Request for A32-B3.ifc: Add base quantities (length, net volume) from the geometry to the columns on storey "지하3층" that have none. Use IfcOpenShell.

First a look at what the model holds.

```python
import ifcopenshell
import ifcopenshell.util.element
import ifcopenshell.util.unit

model = ifcopenshell.open("A32-B3.ifc")
print(model.schema)
for unit_type in ("LENGTHUNIT", "AREAUNIT", "VOLUMEUNIT"):
    print(unit_type, ifcopenshell.util.unit.calculate_unit_scale(model, unit_type))
storey = next(s for s in model.by_type("IfcBuildingStorey") if s.Name == "지하3층")
columns = [e for e in ifcopenshell.util.element.get_decomposition(storey) if e.is_a("IfcColumn")]
for e in sorted(columns, key=lambda e: e.id()):
    print(e.id(), e.is_a(), e.Name, list(ifcopenshell.util.element.get_psets(e, qtos_only=True)), sep=" | ")
```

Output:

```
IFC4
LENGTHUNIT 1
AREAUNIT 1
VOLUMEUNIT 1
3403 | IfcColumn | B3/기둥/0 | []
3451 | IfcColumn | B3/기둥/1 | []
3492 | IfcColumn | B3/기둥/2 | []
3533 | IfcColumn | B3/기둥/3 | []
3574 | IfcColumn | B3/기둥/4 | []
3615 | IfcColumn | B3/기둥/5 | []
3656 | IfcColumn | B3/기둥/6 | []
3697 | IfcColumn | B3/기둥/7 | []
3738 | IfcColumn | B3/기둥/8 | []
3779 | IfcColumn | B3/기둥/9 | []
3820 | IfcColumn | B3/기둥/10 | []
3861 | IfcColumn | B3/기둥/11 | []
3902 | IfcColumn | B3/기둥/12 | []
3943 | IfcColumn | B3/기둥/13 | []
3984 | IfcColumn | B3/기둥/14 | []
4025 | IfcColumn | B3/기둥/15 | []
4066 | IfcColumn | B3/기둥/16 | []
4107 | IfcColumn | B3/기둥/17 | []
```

```python
import ifcopenshell
import ifcopenshell.api.pset
import ifcopenshell.geom
import ifcopenshell.util.element
import ifcopenshell.util.shape
import ifcopenshell.util.unit

model = ifcopenshell.open("A32-B3.ifc")
unit_scale = ifcopenshell.util.unit.calculate_unit_scale(model)
volume_scale = ifcopenshell.util.unit.calculate_unit_scale(model, "VOLUMEUNIT")
settings = ifcopenshell.geom.settings()

storey = next(s for s in model.by_type("IfcBuildingStorey") if s.Name == "지하3층")
columns = [e for e in ifcopenshell.util.element.get_decomposition(storey) if e.is_a("IfcColumn")]

for e in sorted(columns, key=lambda e: e.id()):
    if ifcopenshell.util.element.get_psets(e, qtos_only=True, should_inherit=False):
        continue
    # Geometry comes back in metres, in the element's own axes.
    shape = ifcopenshell.geom.create_shape(settings, e)
    values = {
        "Length": ifcopenshell.util.shape.get_z(shape.geometry) / unit_scale,
        "NetVolume": ifcopenshell.util.shape.get_volume(shape.geometry) / volume_scale,
    }
    qto = ifcopenshell.api.pset.add_qto(model, product=e, name="Qto_ColumnBaseQuantities")
    ifcopenshell.api.pset.edit_qto(model, qto=qto, properties=values)
    print(e.id(), {k: round(v, 3) for k, v in values.items()})

model.write("A32-B3_edited.ifc")
```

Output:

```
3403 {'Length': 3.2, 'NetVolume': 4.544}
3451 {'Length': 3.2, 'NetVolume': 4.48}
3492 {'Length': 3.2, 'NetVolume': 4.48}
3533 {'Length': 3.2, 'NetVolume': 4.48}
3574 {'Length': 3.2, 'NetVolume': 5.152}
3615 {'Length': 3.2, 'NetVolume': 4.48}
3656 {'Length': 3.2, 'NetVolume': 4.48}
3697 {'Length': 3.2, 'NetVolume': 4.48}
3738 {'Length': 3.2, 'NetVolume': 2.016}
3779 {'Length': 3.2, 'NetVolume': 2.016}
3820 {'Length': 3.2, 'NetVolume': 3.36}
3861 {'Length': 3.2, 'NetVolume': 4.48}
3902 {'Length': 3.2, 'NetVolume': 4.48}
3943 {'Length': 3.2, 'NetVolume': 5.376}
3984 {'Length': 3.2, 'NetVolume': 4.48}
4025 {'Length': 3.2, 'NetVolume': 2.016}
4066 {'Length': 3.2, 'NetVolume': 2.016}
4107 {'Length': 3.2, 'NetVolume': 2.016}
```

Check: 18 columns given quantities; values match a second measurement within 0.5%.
